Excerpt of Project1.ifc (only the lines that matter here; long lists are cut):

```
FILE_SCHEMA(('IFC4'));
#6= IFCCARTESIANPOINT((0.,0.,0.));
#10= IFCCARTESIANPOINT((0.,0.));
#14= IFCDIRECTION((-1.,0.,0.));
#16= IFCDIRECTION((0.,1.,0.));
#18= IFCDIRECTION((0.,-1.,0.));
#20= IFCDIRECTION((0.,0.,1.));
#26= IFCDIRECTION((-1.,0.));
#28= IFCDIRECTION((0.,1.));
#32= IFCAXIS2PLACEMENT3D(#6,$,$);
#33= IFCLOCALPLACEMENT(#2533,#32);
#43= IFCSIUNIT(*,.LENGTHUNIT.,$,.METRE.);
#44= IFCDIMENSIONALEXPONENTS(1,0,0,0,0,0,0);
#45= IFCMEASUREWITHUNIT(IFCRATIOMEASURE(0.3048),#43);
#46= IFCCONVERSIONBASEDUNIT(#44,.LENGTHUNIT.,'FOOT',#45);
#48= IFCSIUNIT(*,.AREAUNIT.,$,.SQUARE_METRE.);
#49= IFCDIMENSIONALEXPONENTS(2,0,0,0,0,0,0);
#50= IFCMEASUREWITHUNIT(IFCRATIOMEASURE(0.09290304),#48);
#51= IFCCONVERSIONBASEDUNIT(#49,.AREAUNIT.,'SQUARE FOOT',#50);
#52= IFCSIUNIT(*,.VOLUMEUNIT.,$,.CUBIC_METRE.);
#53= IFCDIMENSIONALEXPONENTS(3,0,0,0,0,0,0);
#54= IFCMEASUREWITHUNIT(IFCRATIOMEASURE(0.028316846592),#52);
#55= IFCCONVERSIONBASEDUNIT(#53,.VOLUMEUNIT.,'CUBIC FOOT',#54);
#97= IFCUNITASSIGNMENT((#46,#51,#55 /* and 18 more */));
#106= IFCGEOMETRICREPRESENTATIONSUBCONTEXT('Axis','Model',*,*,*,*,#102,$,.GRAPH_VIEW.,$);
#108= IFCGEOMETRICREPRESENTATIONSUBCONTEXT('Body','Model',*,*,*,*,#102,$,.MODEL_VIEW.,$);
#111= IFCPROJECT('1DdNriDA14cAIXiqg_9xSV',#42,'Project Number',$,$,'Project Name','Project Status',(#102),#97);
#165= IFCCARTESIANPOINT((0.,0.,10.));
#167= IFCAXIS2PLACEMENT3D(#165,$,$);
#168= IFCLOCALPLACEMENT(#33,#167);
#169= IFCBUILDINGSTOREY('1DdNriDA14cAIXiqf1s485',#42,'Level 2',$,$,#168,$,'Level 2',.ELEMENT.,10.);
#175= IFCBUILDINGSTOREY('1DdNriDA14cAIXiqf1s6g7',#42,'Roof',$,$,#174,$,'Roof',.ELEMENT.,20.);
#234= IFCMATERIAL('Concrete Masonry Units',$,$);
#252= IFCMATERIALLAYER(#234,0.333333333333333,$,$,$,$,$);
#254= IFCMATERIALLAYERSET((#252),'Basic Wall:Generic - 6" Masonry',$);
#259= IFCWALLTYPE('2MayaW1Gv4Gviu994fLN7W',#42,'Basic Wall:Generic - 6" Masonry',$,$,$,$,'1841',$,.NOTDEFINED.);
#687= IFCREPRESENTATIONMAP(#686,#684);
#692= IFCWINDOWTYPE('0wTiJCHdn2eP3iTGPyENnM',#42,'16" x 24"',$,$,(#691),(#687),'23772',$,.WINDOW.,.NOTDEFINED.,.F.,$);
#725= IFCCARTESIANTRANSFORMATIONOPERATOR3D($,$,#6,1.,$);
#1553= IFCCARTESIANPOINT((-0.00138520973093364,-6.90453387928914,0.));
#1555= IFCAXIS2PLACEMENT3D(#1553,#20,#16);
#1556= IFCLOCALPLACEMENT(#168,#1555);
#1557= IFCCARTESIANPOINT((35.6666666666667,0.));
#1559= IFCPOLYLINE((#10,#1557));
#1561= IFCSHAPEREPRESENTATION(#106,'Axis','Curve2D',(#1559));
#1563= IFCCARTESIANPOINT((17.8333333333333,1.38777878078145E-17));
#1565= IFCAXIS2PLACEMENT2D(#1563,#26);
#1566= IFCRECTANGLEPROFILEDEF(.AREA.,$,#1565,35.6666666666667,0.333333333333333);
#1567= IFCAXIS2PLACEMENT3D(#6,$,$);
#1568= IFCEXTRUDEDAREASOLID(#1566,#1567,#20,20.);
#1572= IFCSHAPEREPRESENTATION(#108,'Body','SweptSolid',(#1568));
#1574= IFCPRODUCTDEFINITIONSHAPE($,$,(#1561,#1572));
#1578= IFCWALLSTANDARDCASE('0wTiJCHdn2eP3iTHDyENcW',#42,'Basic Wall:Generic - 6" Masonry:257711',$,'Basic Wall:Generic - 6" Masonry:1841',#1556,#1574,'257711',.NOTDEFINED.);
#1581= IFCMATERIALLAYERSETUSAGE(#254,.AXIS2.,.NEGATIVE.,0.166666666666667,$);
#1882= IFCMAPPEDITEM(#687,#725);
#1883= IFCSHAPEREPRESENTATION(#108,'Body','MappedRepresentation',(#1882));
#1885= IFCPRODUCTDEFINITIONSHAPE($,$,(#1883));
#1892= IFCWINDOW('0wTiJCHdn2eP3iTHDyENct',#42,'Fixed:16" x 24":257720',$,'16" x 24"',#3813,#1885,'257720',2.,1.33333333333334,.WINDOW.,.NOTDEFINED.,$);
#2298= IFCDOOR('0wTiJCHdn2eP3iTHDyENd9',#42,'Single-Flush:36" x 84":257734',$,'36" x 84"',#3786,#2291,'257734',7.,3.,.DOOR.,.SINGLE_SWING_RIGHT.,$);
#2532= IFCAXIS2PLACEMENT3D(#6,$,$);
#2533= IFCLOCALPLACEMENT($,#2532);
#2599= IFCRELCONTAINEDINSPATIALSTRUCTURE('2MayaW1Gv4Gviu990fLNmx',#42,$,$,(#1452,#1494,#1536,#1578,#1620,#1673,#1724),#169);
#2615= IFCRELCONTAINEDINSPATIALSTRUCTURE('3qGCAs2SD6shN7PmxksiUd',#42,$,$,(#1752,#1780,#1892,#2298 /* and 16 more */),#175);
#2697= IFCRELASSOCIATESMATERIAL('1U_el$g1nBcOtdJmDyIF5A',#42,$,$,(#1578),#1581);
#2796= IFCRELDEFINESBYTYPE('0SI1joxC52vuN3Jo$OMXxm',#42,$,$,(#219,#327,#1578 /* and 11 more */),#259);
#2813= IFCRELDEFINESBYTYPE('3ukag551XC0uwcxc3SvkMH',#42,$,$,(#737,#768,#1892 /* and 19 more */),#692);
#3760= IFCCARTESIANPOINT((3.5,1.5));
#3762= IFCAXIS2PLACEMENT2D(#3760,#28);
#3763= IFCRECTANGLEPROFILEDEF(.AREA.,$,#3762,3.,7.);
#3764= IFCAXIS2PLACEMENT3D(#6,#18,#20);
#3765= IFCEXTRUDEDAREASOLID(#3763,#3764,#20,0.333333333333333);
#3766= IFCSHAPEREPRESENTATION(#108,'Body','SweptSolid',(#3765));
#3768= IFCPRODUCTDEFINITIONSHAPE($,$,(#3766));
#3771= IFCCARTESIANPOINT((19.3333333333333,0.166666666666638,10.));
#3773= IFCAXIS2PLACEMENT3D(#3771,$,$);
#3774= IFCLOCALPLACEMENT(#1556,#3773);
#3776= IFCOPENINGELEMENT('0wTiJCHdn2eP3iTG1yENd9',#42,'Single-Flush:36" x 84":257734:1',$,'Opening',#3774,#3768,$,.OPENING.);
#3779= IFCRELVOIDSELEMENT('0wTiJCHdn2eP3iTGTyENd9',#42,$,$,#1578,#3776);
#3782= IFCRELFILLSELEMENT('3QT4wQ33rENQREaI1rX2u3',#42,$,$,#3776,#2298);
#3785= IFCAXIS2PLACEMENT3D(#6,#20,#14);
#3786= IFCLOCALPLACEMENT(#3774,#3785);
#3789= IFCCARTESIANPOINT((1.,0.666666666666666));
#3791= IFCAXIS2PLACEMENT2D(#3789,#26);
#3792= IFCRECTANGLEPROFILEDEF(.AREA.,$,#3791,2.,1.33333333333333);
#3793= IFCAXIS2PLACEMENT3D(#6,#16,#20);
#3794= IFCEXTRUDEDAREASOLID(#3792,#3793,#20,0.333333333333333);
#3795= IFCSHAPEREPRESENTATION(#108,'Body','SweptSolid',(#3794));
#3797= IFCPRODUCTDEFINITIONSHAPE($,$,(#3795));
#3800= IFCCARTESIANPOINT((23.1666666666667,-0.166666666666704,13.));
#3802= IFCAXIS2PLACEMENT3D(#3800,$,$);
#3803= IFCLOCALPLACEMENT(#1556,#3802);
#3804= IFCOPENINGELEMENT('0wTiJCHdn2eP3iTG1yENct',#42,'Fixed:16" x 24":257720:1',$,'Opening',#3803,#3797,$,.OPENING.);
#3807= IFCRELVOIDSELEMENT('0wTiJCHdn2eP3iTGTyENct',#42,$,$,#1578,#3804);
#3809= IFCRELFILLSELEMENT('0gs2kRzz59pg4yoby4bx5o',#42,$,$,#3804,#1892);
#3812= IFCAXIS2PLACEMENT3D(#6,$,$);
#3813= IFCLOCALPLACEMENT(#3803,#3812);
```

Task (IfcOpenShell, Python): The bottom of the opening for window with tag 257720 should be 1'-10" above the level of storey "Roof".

```python
import numpy as np
import ifcopenshell
import ifcopenshell.api.geometry
import ifcopenshell.geom
import ifcopenshell.util.element
import ifcopenshell.util.placement
import ifcopenshell.util.shape
import ifcopenshell.util.unit

model = ifcopenshell.open("Project1.ifc")
unit_scale = ifcopenshell.util.unit.calculate_unit_scale(model)

window = model.by_guid("0wTiJCHdn2eP3iTHDyENct")
opening = window.FillsVoids[0].RelatingOpeningElement
storey = ifcopenshell.util.element.get_container(window, ifc_class="IfcBuildingStorey")
level = ifcopenshell.util.placement.get_local_placement(storey.ObjectPlacement)[2, 3]

# The opening's origin need not be at the sill, so measure its lowest point.
shape = ifcopenshell.geom.create_shape(ifcopenshell.geom.settings(), opening)
bottom = ifcopenshell.util.shape.get_shape_bottom_elevation(shape, shape.geometry) / unit_scale
dz = level + 22 * 0.0254 / unit_scale - bottom

shift = np.array([0.0, 0.0, dz])
# The window is placed relative to its opening, so it follows when the opening moves.
matrix = ifcopenshell.util.placement.get_local_placement(opening.ObjectPlacement)
matrix[:3, 3] += shift
ifcopenshell.api.geometry.edit_object_placement(
    model, product=opening, matrix=matrix, is_si=False, should_transform_children=True
)

print(f"moved by {dz * unit_scale:+.3f} m")

model.write("Project1_rev.ifc")
```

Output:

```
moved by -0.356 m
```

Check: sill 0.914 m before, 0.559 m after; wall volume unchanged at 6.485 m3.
